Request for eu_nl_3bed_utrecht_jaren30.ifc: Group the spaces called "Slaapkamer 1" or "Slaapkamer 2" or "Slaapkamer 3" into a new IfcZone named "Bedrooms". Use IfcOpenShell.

First a look at what the model holds.

```python
import ifcopenshell

model = ifcopenshell.open("eu_nl_3bed_utrecht_jaren30.ifc")
print(model.schema)
seen = {}
for space in model.by_type("IfcSpace"):
    seen[space.LongName] = seen.get(space.LongName, 0) + 1
for name, count in sorted(seen.items(), key=str):
    print(count, "x", name)
print("zones:", [z.Name for z in model.by_type("IfcZone")][:20])
```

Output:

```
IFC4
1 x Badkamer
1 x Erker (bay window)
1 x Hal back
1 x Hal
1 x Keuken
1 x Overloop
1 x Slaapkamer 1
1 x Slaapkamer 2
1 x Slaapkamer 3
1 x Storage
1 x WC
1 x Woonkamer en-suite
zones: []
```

```python
import ifcopenshell
import ifcopenshell.api.group
import ifcopenshell.api.root

model = ifcopenshell.open("eu_nl_3bed_utrecht_jaren30.ifc")

names = {"Slaapkamer 1", "Slaapkamer 2", "Slaapkamer 3"}
spaces = [s for s in model.by_type("IfcSpace") if s.LongName in names]

zone = ifcopenshell.api.root.create_entity(model, ifc_class="IfcZone", name="Bedrooms")
ifcopenshell.api.group.assign_group(model, products=spaces, group=zone)
print(len(spaces), "spaces in", zone.Name)

model.write("eu_nl_3bed_utrecht_jaren30_edited.ifc")
```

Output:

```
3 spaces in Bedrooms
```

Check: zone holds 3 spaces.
